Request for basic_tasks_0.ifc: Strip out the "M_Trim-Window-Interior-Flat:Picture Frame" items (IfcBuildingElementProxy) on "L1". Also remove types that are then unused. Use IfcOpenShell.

First a look at what the model holds.

```python
import ifcopenshell
import ifcopenshell.util.element

model = ifcopenshell.open("basic_tasks_0.ifc")
print(model.schema)
storey = next(s for s in model.by_type("IfcBuildingStorey") if s.Name == "L1")
proxies = [e for e in ifcopenshell.util.element.get_decomposition(storey) if e.is_a("IfcBuildingElementProxy")]
seen = {}
for e in proxies:
    element_type = ifcopenshell.util.element.get_type(e)
    name = element_type.Name if element_type not in (None, e) else None
    seen[name] = seen.get(name, 0) + 1
for name, count in sorted(seen.items(), key=str):
    print(count, "x", name)
```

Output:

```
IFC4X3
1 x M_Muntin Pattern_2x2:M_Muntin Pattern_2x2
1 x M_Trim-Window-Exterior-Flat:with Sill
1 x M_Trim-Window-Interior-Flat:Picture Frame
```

```python
import ifcopenshell
import ifcopenshell.api.root
import ifcopenshell.util.element

model = ifcopenshell.open("basic_tasks_0.ifc")

storey = next(s for s in model.by_type("IfcBuildingStorey") if s.Name == "L1")
proxies = [e for e in ifcopenshell.util.element.get_decomposition(storey) if e.is_a("IfcBuildingElementProxy")]
targets = [e for e in proxies if (t := ifcopenshell.util.element.get_type(e)) not in (None, e) and t.Name == "M_Trim-Window-Interior-Flat:Picture Frame"]
types = {ifcopenshell.util.element.get_type(e) for e in targets} - {None, *targets}

for e in targets:
    ifcopenshell.api.root.remove_product(model, product=e)
print(len(targets), "removed")

unused = [t for t in types if not ifcopenshell.util.element.get_types(t)]
for t in unused:
    ifcopenshell.api.root.remove_product(model, product=t)
print(len(unused), "unused types removed")

model.write("basic_tasks_0_rev.ifc")
```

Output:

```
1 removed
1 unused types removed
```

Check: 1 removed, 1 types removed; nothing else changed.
